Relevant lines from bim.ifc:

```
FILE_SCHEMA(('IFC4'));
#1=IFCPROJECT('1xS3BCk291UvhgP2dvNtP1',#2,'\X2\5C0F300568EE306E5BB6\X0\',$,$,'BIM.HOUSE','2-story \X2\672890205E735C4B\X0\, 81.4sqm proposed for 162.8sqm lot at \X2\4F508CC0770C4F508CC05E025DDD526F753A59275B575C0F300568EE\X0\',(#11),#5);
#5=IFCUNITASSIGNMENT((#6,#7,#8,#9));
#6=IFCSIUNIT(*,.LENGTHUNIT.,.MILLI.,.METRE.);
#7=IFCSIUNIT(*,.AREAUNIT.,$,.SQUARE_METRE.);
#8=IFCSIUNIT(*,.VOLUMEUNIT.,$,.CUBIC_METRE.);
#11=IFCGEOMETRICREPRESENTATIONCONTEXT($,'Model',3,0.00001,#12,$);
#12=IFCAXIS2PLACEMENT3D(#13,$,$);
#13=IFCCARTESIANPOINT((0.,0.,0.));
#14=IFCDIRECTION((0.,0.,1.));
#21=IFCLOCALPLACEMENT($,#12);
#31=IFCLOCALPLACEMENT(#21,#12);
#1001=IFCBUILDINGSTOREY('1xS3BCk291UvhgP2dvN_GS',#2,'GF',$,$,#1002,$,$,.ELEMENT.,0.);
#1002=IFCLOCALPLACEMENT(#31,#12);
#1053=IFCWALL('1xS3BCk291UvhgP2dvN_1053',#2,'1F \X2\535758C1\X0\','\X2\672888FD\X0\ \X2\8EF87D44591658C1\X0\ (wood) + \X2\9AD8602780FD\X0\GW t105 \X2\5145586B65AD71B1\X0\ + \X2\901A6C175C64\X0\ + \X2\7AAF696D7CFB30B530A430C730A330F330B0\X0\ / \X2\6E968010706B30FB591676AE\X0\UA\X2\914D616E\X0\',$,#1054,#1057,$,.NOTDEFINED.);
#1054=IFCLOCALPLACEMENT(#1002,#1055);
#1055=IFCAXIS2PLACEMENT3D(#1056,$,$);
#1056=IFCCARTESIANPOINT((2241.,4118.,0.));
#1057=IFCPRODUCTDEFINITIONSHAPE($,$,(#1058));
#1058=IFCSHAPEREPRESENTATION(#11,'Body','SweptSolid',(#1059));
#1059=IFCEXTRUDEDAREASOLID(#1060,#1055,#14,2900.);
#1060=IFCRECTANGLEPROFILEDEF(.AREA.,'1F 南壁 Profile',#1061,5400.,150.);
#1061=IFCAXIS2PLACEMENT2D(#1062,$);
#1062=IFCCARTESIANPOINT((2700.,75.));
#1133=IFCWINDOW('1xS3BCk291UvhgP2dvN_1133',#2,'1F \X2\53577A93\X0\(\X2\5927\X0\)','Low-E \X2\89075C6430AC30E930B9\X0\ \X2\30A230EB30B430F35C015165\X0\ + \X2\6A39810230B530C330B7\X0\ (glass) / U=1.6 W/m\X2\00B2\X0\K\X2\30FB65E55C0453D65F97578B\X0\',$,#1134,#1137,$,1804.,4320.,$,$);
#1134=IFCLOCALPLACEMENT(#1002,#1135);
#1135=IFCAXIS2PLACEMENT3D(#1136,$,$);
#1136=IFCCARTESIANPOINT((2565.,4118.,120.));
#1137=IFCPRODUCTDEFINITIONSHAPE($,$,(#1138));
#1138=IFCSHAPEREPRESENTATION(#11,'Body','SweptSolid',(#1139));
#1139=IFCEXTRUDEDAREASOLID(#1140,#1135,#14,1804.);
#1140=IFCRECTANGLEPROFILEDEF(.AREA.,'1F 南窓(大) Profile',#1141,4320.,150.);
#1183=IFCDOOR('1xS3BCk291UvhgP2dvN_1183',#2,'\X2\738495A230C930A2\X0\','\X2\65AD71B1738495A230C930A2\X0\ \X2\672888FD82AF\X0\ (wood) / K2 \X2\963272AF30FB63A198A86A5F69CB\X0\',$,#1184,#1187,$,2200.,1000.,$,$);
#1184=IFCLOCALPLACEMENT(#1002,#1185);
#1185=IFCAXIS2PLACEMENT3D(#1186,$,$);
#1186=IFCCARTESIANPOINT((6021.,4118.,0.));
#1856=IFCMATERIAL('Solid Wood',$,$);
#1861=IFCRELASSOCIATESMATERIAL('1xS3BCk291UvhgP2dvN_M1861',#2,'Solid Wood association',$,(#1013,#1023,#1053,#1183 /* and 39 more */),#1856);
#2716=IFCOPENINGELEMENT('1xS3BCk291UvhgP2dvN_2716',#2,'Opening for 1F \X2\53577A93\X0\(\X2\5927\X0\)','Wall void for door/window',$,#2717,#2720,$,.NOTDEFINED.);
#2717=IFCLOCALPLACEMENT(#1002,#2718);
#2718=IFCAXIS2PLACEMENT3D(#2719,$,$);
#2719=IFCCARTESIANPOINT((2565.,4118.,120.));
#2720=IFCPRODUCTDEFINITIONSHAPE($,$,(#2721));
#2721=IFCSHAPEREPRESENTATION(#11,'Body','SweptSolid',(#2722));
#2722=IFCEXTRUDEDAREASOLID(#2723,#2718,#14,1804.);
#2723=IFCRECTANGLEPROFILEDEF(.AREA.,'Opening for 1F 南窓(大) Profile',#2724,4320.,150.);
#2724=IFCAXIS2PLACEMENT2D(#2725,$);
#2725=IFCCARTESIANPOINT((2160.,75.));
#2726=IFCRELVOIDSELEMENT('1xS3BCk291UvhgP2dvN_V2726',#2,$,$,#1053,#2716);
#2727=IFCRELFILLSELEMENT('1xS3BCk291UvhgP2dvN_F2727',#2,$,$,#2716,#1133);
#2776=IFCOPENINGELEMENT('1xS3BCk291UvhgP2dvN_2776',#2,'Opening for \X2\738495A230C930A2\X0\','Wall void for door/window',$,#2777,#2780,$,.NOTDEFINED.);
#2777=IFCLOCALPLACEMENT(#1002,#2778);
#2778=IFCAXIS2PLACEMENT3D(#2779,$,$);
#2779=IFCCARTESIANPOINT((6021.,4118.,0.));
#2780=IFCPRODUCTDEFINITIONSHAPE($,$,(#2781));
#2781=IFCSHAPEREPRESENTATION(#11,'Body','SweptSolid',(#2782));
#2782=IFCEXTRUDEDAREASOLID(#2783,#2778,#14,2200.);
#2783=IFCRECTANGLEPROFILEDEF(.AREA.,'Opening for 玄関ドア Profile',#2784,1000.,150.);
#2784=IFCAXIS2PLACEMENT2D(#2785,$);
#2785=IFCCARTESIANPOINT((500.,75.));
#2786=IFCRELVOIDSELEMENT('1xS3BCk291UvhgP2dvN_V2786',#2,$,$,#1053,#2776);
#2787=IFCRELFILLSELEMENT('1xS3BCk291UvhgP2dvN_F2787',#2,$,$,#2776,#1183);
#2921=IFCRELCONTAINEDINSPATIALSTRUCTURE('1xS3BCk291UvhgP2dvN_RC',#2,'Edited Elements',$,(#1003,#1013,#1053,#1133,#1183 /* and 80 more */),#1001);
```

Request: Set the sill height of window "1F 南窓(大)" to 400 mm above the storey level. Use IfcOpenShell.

```python
import numpy as np
import ifcopenshell
import ifcopenshell.api.geometry
import ifcopenshell.geom
import ifcopenshell.util.element
import ifcopenshell.util.placement
import ifcopenshell.util.shape
import ifcopenshell.util.unit

model = ifcopenshell.open("bim.ifc")
unit_scale = ifcopenshell.util.unit.calculate_unit_scale(model)

window = model.by_id(1133)
opening = window.FillsVoids[0].RelatingOpeningElement
storey = ifcopenshell.util.element.get_container(window, ifc_class="IfcBuildingStorey")
level = ifcopenshell.util.placement.get_local_placement(storey.ObjectPlacement)[2, 3]

# The opening's origin need not be at the sill, so measure its lowest point.
shape = ifcopenshell.geom.create_shape(ifcopenshell.geom.settings(), opening)
bottom = ifcopenshell.util.shape.get_shape_bottom_elevation(shape, shape.geometry) / unit_scale
dz = level + 0.4 / unit_scale - bottom

shift = np.array([0.0, 0.0, dz])
# The window is not placed relative to its opening, so move both.
for product in (opening, window):
    matrix = ifcopenshell.util.placement.get_local_placement(product.ObjectPlacement)
    matrix[:3, 3] += shift
    ifcopenshell.api.geometry.edit_object_placement(model, product=product, matrix=matrix, is_si=False)

print(f"moved by {dz * unit_scale:+.3f} m")

model.write("bim_edited.ifc")
```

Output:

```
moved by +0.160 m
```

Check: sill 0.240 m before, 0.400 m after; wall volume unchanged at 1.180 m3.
